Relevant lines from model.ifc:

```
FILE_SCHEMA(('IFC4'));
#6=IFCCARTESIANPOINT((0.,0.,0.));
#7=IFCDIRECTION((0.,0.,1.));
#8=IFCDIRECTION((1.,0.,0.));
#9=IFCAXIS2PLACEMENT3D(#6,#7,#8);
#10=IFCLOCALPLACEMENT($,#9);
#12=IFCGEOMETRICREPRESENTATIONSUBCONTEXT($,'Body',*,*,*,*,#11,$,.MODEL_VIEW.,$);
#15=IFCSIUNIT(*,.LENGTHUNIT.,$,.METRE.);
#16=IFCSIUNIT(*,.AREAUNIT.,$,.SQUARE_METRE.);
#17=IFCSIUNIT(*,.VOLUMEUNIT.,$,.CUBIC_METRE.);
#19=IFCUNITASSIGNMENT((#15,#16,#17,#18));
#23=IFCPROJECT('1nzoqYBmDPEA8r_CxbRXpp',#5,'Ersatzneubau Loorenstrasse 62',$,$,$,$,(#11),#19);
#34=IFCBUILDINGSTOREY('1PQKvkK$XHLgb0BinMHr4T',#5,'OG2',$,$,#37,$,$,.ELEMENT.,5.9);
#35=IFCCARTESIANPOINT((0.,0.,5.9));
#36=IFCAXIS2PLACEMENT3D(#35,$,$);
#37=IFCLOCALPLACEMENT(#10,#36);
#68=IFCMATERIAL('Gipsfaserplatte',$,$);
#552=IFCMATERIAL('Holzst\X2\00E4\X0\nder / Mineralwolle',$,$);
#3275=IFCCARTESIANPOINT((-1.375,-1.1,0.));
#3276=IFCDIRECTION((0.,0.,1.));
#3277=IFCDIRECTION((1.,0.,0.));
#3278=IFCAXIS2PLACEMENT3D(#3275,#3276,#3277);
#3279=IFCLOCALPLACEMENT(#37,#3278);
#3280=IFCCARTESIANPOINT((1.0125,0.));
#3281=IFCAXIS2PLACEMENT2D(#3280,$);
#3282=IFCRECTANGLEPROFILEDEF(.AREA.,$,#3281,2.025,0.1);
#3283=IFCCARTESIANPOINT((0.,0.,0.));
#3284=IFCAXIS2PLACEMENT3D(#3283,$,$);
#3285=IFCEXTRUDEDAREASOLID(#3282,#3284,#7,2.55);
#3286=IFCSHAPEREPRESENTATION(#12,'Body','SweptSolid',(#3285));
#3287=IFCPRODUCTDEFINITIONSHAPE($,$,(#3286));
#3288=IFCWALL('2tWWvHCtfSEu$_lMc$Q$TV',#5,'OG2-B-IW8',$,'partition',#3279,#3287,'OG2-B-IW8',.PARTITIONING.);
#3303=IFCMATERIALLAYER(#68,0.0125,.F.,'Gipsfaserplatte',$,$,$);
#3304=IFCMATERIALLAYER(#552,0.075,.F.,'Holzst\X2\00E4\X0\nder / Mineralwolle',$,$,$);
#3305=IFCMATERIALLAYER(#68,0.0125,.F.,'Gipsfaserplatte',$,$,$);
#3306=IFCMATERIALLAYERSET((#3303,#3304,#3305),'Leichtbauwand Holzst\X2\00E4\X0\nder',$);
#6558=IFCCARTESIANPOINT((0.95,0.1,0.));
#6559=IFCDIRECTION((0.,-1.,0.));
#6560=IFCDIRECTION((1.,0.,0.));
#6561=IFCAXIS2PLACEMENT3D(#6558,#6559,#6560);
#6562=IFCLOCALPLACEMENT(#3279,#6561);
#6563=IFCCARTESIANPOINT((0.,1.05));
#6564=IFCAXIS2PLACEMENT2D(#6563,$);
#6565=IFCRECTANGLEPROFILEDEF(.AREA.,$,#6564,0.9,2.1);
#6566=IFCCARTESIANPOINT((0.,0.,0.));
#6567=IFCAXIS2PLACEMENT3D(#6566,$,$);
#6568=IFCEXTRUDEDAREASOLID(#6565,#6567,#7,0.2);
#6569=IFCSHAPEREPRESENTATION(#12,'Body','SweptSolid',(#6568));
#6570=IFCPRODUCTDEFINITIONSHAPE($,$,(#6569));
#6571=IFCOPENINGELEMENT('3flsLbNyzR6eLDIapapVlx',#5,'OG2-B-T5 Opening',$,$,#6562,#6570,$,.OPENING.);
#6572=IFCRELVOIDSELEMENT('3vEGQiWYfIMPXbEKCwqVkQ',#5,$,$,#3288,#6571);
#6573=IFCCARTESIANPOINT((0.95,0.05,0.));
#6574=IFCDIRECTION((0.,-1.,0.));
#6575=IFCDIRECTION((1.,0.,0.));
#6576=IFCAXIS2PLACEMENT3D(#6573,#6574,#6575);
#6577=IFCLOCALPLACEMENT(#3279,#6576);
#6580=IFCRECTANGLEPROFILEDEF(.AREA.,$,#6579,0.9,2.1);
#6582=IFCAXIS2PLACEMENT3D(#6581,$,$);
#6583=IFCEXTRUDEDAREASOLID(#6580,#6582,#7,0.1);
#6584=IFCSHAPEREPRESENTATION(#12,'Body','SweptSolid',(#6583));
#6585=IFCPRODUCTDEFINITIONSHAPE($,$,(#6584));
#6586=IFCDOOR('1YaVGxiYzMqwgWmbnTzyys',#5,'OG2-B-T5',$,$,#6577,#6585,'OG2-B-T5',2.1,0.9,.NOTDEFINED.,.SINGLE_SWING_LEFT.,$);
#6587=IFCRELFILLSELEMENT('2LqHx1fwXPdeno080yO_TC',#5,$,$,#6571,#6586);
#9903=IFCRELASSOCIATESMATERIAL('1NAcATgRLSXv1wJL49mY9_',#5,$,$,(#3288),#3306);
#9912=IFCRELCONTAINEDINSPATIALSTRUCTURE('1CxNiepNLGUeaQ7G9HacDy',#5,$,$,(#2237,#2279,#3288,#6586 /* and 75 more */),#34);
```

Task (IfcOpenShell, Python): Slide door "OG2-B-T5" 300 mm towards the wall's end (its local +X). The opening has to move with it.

```python
import ifcopenshell
import ifcopenshell.api.geometry
import ifcopenshell.util.placement
import ifcopenshell.util.unit

model = ifcopenshell.open("model.ifc")
unit_scale = ifcopenshell.util.unit.calculate_unit_scale(model)

door = model.by_guid("1YaVGxiYzMqwgWmbnTzyys")
opening = door.FillsVoids[0].RelatingOpeningElement
wall = opening.VoidsElements[0].RelatingBuildingElement

wall_matrix = ifcopenshell.util.placement.get_local_placement(wall.ObjectPlacement)
shift = wall_matrix[:3, 0] * 0.3 / unit_scale
before = ifcopenshell.util.placement.get_local_placement(door.ObjectPlacement)[:3, 3].copy()

# The door is not placed relative to its opening, so move both.
for product in (opening, door):
    matrix = ifcopenshell.util.placement.get_local_placement(product.ObjectPlacement)
    matrix[:3, 3] += shift
    ifcopenshell.api.geometry.edit_object_placement(model, product=product, matrix=matrix, is_si=False)

after = ifcopenshell.util.placement.get_local_placement(door.ObjectPlacement)[:3, 3]
print("door moved by", (after - before).round(3) + 0.0)

model.write("model_v2.ifc")
```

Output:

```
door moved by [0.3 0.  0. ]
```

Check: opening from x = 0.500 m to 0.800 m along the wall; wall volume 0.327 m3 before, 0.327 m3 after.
